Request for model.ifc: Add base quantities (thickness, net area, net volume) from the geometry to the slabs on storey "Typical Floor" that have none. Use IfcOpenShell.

First a look at what the model holds.

```python
import ifcopenshell
import ifcopenshell.util.element
import ifcopenshell.util.unit

model = ifcopenshell.open("model.ifc")
print(model.schema)
for unit_type in ("LENGTHUNIT", "AREAUNIT", "VOLUMEUNIT"):
    print(unit_type, ifcopenshell.util.unit.calculate_unit_scale(model, unit_type))
storey = next(s for s in model.by_type("IfcBuildingStorey") if s.Name == "Typical Floor")
slabs = [e for e in ifcopenshell.util.element.get_decomposition(storey) if e.is_a("IfcSlab")]
for e in sorted(slabs, key=lambda e: e.id()):
    print(e.id(), e.is_a(), e.Name, list(ifcopenshell.util.element.get_psets(e, qtos_only=True)), sep=" | ")
```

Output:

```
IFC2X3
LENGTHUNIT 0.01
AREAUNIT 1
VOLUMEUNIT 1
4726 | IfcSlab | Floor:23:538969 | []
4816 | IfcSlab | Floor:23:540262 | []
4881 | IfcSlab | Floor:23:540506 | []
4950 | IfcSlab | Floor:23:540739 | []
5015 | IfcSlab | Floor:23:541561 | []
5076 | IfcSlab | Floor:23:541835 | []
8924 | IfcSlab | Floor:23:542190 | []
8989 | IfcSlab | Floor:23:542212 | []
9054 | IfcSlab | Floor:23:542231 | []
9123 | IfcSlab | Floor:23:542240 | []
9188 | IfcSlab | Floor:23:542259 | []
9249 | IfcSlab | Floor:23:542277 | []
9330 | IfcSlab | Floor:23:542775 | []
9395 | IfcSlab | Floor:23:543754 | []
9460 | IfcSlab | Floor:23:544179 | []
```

```python
import ifcopenshell
import ifcopenshell.api.pset
import ifcopenshell.geom
import ifcopenshell.util.element
import ifcopenshell.util.shape
import ifcopenshell.util.unit

model = ifcopenshell.open("model.ifc")
unit_scale = ifcopenshell.util.unit.calculate_unit_scale(model)
area_scale = ifcopenshell.util.unit.calculate_unit_scale(model, "AREAUNIT")
volume_scale = ifcopenshell.util.unit.calculate_unit_scale(model, "VOLUMEUNIT")
settings = ifcopenshell.geom.settings()

storey = next(s for s in model.by_type("IfcBuildingStorey") if s.Name == "Typical Floor")
slabs = [e for e in ifcopenshell.util.element.get_decomposition(storey) if e.is_a("IfcSlab")]

for e in sorted(slabs, key=lambda e: e.id()):
    if ifcopenshell.util.element.get_psets(e, qtos_only=True, should_inherit=False):
        continue
    # Geometry comes back in metres, in the element's own axes.
    shape = ifcopenshell.geom.create_shape(settings, e)
    values = {
        "Width": ifcopenshell.util.shape.get_z(shape.geometry) / unit_scale,
        "NetArea": ifcopenshell.util.shape.get_footprint_area(shape.geometry) / area_scale,
        "NetVolume": ifcopenshell.util.shape.get_volume(shape.geometry) / volume_scale,
    }
    qto = ifcopenshell.api.pset.add_qto(model, product=e, name="BaseQuantities")
    ifcopenshell.api.pset.edit_qto(model, qto=qto, properties=values)
    print(e.id(), {k: round(v, 3) for k, v in values.items()})

model.write("model_edited.ifc")
```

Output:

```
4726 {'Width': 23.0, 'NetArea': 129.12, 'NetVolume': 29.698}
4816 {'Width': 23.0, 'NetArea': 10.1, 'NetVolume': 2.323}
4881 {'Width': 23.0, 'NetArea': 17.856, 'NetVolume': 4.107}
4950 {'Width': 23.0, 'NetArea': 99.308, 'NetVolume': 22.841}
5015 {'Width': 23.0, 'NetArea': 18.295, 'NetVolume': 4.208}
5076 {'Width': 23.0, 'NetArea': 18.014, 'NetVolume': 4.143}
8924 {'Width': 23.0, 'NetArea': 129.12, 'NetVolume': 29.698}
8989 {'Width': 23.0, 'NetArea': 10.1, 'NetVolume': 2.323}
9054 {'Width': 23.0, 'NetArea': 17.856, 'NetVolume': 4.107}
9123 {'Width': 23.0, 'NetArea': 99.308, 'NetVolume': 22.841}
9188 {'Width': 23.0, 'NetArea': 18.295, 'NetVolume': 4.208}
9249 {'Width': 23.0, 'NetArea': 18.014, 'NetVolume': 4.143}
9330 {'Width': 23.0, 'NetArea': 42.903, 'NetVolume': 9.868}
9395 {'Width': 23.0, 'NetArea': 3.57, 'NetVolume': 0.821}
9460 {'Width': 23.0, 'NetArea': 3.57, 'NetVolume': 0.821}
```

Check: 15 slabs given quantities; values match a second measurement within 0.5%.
